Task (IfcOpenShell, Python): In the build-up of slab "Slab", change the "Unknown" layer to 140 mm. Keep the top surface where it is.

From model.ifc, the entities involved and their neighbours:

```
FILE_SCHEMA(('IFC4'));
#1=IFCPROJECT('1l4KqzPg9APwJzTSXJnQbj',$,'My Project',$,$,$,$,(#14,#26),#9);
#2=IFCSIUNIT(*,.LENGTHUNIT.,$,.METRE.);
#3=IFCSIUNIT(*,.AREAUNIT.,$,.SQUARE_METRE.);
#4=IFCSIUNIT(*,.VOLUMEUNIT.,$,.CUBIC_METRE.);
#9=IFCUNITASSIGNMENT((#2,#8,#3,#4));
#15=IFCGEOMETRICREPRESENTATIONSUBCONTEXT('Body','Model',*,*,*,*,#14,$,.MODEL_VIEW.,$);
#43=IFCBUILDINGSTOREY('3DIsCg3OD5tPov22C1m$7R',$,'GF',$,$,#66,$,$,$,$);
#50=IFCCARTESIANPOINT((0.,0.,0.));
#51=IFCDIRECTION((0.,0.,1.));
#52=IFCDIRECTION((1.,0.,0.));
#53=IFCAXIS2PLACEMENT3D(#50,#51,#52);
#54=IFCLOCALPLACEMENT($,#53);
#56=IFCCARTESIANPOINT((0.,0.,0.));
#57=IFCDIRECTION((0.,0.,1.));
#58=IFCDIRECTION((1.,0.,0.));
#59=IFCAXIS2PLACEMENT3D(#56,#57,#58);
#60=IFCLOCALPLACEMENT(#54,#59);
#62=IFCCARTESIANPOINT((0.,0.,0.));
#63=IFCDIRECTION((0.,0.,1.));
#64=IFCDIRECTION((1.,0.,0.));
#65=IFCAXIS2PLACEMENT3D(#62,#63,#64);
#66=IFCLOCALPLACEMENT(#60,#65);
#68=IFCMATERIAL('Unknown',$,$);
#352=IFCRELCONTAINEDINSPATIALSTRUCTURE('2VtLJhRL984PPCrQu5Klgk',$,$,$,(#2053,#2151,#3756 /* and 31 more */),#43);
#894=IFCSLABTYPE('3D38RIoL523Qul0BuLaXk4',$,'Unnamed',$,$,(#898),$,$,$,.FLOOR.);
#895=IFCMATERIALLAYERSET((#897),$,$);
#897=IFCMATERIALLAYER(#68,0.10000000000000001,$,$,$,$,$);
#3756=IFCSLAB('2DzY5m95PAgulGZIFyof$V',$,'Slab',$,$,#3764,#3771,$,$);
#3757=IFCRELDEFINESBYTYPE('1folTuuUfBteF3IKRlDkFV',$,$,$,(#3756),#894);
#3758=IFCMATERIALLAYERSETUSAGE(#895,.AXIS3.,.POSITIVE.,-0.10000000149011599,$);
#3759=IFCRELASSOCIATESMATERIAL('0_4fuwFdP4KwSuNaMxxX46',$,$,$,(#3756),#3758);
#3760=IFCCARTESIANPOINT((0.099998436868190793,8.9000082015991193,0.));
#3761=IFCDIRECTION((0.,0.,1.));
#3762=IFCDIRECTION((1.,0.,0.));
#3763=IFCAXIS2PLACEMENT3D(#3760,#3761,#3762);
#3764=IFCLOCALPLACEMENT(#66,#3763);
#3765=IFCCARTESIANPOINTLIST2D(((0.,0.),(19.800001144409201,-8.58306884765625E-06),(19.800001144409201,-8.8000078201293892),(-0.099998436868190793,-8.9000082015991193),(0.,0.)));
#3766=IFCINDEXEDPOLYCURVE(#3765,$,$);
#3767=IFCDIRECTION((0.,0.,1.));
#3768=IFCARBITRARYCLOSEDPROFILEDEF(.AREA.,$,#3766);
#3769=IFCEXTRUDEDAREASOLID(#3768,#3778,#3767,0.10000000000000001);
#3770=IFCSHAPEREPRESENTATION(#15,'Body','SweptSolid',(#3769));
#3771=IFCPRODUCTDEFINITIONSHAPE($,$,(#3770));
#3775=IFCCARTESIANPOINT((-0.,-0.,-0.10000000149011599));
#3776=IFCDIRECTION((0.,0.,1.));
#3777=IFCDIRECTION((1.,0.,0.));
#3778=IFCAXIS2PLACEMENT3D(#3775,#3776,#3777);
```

```python
import ifcopenshell
import ifcopenshell.util.element
import ifcopenshell.util.representation

model = ifcopenshell.open("model.ifc")

layer_set = model.by_id(895)
layer = next(l for l in layer_set.MaterialLayers if l.Material and l.Material.Name == "Unknown")
change = 0.14 - layer.LayerThickness
layer.LayerThickness += change

# Geometry does not follow the layer set by itself.
slabs = [e for e in ifcopenshell.util.element.get_elements_by_material(model, layer_set) if e.is_a("IfcSlab")]
for slab in sorted(slabs, key=lambda e: e.id()):
    body = ifcopenshell.util.representation.get_representation(slab, "Model", "Body")
    solid = body.Items[0]
    old_depth = solid.Depth
    solid.Depth += change
    # Extruded upwards: lower the start of the extrusion so the top stays.
    x, y, z = solid.Position.Location.Coordinates
    solid.Position.Location = model.createIfcCartesianPoint((x, y, z - change))
    print(slab.id(), f"{old_depth:g} -> {solid.Depth:g}")

# The layers are counted up from the underside, which has moved.
for usage in {ifcopenshell.util.element.get_material(slab) for slab in slabs}:
    usage.OffsetFromReferenceLine -= change

model.write("model_edited.ifc")
```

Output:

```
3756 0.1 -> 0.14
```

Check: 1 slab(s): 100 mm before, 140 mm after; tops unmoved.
